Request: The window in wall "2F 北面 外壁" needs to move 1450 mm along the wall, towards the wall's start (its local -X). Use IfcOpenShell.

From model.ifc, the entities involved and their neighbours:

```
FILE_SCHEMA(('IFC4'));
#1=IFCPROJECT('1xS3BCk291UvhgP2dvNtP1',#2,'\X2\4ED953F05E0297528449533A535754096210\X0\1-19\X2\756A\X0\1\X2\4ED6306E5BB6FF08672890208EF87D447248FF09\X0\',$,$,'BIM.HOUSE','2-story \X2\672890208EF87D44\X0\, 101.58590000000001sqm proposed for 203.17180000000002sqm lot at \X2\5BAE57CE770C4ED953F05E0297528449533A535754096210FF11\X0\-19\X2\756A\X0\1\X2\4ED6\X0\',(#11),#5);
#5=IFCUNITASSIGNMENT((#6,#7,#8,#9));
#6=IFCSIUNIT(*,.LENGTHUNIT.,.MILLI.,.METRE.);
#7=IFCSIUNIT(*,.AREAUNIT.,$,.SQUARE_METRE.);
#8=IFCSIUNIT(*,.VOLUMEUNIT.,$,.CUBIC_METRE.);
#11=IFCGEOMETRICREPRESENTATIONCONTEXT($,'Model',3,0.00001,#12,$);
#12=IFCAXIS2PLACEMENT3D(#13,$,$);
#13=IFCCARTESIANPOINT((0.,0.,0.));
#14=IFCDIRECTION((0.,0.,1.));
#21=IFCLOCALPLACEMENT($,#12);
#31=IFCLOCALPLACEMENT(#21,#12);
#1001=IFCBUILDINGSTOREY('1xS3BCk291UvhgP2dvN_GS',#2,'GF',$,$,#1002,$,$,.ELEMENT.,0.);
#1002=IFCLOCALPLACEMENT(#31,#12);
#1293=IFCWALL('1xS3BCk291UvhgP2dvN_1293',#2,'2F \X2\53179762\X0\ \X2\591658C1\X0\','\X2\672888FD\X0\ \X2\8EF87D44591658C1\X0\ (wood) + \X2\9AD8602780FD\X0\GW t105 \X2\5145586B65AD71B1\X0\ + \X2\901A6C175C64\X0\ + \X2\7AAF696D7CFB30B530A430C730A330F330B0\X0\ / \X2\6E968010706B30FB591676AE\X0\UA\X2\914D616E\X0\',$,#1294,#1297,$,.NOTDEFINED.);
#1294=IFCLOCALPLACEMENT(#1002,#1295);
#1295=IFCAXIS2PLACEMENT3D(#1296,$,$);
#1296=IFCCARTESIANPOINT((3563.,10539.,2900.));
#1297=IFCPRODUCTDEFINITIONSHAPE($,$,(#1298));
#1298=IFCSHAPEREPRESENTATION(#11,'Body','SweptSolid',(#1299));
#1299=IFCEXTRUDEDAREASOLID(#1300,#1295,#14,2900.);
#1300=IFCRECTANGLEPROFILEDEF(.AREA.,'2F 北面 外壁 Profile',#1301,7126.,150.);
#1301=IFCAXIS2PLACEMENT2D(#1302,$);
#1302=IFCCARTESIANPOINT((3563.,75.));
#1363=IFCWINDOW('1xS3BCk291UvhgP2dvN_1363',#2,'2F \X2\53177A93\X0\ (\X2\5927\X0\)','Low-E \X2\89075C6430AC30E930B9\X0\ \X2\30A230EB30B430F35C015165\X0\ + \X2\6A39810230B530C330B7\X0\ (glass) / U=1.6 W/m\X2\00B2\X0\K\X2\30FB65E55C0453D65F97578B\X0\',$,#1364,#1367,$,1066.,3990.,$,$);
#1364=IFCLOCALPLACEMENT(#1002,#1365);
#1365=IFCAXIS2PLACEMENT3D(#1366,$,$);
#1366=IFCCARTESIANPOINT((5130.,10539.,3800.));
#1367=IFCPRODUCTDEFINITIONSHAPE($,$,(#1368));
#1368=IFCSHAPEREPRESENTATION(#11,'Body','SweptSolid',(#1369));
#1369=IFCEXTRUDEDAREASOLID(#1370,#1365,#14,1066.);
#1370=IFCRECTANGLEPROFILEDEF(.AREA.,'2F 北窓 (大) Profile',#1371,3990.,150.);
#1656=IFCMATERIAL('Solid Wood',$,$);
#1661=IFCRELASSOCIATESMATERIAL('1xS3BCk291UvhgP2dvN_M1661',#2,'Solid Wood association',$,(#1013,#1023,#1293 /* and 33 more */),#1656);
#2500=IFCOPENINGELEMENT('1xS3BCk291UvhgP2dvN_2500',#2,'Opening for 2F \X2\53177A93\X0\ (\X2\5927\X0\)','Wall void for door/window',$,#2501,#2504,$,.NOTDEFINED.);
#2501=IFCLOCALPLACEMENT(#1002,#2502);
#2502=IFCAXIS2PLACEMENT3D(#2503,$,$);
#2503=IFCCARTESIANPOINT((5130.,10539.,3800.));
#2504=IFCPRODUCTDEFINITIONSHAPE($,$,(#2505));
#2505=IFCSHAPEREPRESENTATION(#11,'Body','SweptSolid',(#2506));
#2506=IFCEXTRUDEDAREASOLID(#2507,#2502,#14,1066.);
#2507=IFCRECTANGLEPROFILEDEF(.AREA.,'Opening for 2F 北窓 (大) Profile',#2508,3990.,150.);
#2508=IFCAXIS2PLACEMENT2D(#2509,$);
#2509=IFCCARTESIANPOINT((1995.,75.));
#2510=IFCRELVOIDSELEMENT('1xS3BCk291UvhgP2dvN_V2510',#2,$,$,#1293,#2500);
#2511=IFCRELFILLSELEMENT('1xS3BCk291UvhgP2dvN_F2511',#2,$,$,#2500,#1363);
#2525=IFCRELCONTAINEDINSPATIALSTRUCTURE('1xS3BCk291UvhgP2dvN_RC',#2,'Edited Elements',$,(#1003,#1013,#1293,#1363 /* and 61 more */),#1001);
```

```python
import ifcopenshell
import ifcopenshell.api.geometry
import ifcopenshell.util.placement
import ifcopenshell.util.unit

model = ifcopenshell.open("model.ifc")
unit_scale = ifcopenshell.util.unit.calculate_unit_scale(model)

window = model.by_guid("1xS3BCk291UvhgP2dvN_1363")
opening = window.FillsVoids[0].RelatingOpeningElement
wall = opening.VoidsElements[0].RelatingBuildingElement

wall_matrix = ifcopenshell.util.placement.get_local_placement(wall.ObjectPlacement)
shift = wall_matrix[:3, 0] * -1.45 / unit_scale
before = ifcopenshell.util.placement.get_local_placement(window.ObjectPlacement)[:3, 3].copy()

# The window is not placed relative to its opening, so move both.
for product in (opening, window):
    matrix = ifcopenshell.util.placement.get_local_placement(product.ObjectPlacement)
    matrix[:3, 3] += shift
    ifcopenshell.api.geometry.edit_object_placement(model, product=product, matrix=matrix, is_si=False)

after = ifcopenshell.util.placement.get_local_placement(window.ObjectPlacement)[:3, 3]
print("window moved by", (after - before).round(3) + 0.0)

model.write("model_v2.ifc")
```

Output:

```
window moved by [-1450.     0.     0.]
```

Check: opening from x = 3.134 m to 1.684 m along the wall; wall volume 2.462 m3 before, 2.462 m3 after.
